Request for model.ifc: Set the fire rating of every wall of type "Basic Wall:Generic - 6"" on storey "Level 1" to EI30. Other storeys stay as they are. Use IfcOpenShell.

First a look at what the model holds.

```python
import ifcopenshell
import ifcopenshell.util.element

model = ifcopenshell.open("model.ifc")
print(model.schema)
storey = next(s for s in model.by_type("IfcBuildingStorey") if s.Name == "Level 1")
walls = [e for e in ifcopenshell.util.element.get_decomposition(storey) if e.is_a("IfcWall")]
seen = {}
for e in walls:
    element_type = ifcopenshell.util.element.get_type(e)
    key = (element_type.Name if element_type != e and element_type else None, ifcopenshell.util.element.get_pset(e, "Pset_WallCommon", "FireRating"))
    seen[key] = seen.get(key, 0) + 1
for (name, value), count in sorted(seen.items(), key=str):
    print(count, "x", name, "|", value)
```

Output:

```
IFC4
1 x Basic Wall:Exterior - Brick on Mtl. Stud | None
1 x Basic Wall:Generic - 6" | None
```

```python
import ifcopenshell
import ifcopenshell.api.pset
import ifcopenshell.util.element

model = ifcopenshell.open("model.ifc")

storey = next(s for s in model.by_type("IfcBuildingStorey") if s.Name == "Level 1")
walls = [e for e in ifcopenshell.util.element.get_decomposition(storey) if e.is_a("IfcWall")]

count = 0
for e in walls:
    element_type = ifcopenshell.util.element.get_type(e)
    if element_type in (None, e) or element_type.Name != 'Basic Wall:Generic - 6"':
        continue
    # add_pset returns the element's existing set when there is one.
    pset = ifcopenshell.api.pset.add_pset(model, product=e, name="Pset_WallCommon")
    ifcopenshell.api.pset.edit_pset(model, pset=pset, properties={"FireRating": "EI30"})
    count += 1

print(count, "walls updated")

model.write("model-out.ifc")
```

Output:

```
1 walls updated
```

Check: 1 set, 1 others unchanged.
